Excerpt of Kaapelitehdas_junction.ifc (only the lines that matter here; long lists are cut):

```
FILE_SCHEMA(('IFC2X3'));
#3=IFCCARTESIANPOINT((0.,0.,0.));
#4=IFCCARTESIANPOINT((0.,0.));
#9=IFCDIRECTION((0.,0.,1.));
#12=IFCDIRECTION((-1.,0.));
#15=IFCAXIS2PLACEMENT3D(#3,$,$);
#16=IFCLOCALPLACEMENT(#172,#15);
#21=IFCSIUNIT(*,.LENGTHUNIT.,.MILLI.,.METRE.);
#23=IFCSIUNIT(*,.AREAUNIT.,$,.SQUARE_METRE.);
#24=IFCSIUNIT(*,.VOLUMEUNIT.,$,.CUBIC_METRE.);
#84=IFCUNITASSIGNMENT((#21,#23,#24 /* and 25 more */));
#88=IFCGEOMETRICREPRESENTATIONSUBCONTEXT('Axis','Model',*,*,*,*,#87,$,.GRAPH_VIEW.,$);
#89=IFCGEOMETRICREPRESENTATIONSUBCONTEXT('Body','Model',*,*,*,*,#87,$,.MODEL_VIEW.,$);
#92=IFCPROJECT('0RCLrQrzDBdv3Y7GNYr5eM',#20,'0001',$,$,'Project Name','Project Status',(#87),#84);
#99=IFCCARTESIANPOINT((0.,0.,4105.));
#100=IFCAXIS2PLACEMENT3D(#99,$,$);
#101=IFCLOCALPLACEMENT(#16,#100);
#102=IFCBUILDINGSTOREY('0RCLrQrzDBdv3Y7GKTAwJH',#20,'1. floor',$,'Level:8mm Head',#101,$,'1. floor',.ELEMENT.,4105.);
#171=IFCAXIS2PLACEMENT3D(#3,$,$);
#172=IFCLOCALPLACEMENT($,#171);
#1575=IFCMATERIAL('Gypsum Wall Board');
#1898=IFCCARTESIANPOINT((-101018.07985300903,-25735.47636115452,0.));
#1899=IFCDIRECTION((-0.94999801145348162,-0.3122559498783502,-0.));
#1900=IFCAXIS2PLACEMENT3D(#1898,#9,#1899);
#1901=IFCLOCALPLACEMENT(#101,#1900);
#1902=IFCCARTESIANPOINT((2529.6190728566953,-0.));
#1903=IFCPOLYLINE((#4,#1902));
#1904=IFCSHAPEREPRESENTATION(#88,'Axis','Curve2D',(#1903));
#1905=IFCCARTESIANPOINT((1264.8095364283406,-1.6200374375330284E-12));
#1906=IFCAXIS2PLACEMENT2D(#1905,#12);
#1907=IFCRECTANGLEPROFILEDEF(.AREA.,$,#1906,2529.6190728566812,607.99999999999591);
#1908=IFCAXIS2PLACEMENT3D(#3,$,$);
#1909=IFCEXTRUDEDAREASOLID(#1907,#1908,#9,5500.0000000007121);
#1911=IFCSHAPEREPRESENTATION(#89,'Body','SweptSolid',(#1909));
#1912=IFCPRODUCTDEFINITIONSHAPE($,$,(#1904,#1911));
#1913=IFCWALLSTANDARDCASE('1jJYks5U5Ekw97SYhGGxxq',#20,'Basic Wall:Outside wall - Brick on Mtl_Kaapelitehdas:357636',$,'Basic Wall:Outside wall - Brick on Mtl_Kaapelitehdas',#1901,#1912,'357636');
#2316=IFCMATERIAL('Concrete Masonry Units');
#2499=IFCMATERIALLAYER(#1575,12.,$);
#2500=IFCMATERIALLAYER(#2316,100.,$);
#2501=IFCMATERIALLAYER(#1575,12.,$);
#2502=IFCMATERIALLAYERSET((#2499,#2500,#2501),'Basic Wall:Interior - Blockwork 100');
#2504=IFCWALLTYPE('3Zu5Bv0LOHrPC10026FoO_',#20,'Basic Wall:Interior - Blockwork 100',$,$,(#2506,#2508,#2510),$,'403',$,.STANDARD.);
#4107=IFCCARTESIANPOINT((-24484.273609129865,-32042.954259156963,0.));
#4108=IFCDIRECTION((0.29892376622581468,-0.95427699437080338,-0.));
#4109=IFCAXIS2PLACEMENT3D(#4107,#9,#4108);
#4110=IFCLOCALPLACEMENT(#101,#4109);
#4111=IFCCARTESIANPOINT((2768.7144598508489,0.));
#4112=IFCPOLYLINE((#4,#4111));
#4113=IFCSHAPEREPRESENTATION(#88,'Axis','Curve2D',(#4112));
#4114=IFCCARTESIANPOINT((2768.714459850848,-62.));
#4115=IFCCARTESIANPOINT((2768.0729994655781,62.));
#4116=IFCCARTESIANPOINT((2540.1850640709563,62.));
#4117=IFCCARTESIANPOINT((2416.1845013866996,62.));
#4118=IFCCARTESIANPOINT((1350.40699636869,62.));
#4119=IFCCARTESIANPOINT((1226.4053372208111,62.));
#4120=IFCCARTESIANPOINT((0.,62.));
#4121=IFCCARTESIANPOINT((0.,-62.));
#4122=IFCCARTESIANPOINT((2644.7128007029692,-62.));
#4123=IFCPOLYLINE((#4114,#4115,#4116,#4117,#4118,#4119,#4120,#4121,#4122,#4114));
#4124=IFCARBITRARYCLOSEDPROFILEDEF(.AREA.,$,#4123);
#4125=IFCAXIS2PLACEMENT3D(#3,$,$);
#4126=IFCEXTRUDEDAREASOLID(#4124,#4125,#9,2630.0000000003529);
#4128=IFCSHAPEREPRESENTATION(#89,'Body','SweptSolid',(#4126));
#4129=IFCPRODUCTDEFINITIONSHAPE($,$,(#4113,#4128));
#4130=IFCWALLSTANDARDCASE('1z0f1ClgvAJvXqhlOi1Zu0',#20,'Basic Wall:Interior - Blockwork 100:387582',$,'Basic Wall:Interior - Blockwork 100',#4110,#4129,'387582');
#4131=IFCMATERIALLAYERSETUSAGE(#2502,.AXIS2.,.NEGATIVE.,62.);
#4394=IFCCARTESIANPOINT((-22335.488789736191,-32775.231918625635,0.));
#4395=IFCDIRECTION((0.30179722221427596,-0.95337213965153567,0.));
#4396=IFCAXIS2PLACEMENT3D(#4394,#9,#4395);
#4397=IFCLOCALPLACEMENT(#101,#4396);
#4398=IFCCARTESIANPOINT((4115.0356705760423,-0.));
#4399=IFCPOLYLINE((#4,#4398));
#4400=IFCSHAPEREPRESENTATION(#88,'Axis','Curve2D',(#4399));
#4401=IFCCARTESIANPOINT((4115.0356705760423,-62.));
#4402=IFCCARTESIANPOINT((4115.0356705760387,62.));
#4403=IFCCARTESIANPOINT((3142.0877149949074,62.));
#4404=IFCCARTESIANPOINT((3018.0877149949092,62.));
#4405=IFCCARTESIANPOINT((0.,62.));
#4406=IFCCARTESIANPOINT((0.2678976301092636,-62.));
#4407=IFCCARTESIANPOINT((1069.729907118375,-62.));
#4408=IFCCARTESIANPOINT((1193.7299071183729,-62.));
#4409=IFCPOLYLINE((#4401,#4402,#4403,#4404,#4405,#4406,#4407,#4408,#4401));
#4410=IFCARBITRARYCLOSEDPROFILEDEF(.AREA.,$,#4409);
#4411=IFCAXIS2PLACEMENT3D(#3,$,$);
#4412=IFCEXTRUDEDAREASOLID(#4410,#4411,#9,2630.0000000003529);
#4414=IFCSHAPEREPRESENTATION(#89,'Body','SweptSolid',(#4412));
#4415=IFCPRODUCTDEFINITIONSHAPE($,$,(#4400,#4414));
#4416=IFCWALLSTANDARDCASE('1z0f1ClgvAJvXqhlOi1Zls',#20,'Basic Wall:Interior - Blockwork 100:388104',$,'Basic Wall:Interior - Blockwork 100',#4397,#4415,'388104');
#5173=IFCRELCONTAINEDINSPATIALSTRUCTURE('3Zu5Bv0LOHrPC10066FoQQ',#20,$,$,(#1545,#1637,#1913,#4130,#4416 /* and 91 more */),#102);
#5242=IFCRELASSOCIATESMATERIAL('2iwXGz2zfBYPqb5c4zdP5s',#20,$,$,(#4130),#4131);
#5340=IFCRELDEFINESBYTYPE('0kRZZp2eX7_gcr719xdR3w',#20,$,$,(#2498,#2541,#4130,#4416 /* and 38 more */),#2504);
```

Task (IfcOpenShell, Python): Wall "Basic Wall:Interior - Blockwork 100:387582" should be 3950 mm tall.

```python
import ifcopenshell
import ifcopenshell.geom
import ifcopenshell.util.representation
import ifcopenshell.util.shape
import ifcopenshell.util.unit

model = ifcopenshell.open("Kaapelitehdas_junction.ifc")
unit_scale = ifcopenshell.util.unit.calculate_unit_scale(model)
settings = ifcopenshell.geom.settings()


def volume(element):
    """Net volume in cubic metres, openings subtracted."""
    shape = ifcopenshell.geom.create_shape(settings, element)
    return ifcopenshell.util.shape.get_volume(shape.geometry)


wall = model.by_guid("1z0f1ClgvAJvXqhlOi1Zu0")
before = volume(wall)

body = ifcopenshell.util.representation.get_representation(wall, "Model", "Body")
solid = body.Items[0]
old_height = solid.Depth
solid.Depth = 3.95 / unit_scale
after = volume(wall)

print(f"height {old_height:g} -> {solid.Depth:g}, volume {before:.3f} -> {after:.3f} m3")

model.write("Kaapelitehdas_junction-out.ifc")
```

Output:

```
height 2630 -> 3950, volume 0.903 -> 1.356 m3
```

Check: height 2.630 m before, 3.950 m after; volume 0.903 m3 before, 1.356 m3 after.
